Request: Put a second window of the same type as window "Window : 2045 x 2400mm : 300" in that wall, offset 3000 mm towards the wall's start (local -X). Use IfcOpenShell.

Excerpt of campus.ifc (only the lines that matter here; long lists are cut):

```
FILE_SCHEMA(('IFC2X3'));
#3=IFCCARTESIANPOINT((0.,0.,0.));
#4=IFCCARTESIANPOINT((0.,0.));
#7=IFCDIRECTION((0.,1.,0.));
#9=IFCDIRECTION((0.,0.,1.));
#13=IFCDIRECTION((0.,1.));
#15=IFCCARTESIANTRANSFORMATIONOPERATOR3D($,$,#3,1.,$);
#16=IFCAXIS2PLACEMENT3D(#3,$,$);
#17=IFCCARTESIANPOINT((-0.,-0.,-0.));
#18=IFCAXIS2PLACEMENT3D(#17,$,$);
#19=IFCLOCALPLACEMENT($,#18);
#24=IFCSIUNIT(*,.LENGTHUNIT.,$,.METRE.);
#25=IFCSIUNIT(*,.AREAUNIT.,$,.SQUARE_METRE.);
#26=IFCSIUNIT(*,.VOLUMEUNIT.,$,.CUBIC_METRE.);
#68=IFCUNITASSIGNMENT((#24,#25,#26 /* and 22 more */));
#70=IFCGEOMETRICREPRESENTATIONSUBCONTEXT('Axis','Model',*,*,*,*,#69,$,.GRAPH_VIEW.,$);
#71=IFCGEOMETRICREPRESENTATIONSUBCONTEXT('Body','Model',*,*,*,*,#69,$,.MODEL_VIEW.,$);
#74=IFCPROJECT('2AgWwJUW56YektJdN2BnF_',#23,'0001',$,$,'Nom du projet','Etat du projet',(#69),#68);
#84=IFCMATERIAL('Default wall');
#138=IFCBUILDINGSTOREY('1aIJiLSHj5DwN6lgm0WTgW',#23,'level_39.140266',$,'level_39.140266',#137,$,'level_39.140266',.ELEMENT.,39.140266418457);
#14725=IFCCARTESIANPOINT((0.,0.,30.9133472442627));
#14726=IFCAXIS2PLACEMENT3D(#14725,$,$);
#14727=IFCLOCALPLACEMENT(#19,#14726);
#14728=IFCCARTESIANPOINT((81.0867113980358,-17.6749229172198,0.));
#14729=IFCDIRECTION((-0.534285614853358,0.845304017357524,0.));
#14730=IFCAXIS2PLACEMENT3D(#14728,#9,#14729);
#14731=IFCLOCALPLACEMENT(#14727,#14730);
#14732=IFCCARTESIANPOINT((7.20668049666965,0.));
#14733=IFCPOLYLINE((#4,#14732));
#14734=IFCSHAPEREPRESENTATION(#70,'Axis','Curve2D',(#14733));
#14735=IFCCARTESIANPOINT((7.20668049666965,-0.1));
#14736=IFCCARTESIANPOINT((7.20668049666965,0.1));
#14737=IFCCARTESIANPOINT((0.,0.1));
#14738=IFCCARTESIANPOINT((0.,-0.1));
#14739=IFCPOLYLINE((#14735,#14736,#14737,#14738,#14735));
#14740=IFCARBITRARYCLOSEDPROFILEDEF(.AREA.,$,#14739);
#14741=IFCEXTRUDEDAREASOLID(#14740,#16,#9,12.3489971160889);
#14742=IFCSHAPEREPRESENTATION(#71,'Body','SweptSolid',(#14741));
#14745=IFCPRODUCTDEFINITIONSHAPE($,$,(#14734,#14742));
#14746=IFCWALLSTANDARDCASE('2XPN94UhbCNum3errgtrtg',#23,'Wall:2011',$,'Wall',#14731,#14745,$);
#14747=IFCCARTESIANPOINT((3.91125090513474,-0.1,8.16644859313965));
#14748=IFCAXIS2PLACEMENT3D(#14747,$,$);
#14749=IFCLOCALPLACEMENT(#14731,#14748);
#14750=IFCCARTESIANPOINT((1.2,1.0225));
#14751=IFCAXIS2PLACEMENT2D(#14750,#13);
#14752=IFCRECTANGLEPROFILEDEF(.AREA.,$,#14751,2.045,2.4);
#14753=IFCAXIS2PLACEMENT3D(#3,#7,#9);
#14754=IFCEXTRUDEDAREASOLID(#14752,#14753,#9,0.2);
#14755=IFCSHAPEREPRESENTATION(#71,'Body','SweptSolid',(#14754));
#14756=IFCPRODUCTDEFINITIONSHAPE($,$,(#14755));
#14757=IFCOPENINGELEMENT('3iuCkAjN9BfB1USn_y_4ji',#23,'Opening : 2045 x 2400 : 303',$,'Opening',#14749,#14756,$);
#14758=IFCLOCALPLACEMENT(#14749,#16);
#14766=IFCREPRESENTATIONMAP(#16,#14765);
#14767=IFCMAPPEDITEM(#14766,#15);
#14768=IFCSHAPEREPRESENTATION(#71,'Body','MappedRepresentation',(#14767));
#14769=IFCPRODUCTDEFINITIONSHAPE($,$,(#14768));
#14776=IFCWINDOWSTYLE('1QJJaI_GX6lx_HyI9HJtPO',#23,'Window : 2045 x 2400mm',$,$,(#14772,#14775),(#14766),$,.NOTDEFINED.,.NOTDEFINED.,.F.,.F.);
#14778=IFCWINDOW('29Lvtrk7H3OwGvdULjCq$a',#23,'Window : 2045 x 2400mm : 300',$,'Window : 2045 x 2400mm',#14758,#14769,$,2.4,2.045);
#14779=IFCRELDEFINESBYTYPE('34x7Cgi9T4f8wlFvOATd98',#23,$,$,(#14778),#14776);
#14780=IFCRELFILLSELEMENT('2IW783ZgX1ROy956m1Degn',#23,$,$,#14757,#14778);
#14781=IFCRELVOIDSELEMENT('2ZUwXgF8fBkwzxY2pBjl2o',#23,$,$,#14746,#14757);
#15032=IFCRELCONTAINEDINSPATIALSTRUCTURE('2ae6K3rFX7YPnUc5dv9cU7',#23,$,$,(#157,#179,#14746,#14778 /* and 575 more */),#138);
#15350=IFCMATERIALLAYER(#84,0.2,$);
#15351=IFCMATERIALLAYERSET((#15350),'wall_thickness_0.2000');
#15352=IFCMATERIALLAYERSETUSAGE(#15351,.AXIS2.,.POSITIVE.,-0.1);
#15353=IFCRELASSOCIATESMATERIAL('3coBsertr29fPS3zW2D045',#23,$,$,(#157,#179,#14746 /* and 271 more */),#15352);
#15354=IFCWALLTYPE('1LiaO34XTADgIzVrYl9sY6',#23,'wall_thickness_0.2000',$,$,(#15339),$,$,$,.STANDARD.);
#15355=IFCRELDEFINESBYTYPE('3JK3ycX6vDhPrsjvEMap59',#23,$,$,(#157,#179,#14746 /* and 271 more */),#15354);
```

```python
import ifcopenshell
import ifcopenshell.api.feature
import ifcopenshell.api.geometry
import ifcopenshell.api.root
import ifcopenshell.geom
import ifcopenshell.util.element
import ifcopenshell.util.placement
import ifcopenshell.util.shape
import ifcopenshell.util.unit

model = ifcopenshell.open("campus.ifc")
unit_scale = ifcopenshell.util.unit.calculate_unit_scale(model)
settings = ifcopenshell.geom.settings()


def volume(element):
    """Net volume in cubic metres, openings subtracted."""
    shape = ifcopenshell.geom.create_shape(settings, element)
    return ifcopenshell.util.shape.get_volume(shape.geometry)


window = model.by_guid("29Lvtrk7H3OwGvdULjCq$a")
opening = window.FillsVoids[0].RelatingOpeningElement
wall = opening.VoidsElements[0].RelatingBuildingElement
before = volume(wall)
shift = ifcopenshell.util.placement.get_local_placement(wall.ObjectPlacement)[:3, 0] * -3 / unit_scale

# copy_class copies the void relationship, type, container and properties, but no geometry.
new_opening = ifcopenshell.api.root.copy_class(model, product=opening)
new_opening.Representation = ifcopenshell.util.element.copy_deep(
    model, opening.Representation, exclude=["IfcGeometricRepresentationContext", "IfcRepresentationMap"]
)
new_opening.Name = "Opening : 2045 x 2400"
new_window = ifcopenshell.api.root.copy_class(model, product=window)
new_window.Representation = ifcopenshell.util.element.copy_deep(
    model, window.Representation, exclude=["IfcGeometricRepresentationContext", "IfcRepresentationMap"]
)
new_window.Name = "Window : 2045 x 2400mm"
fills = ifcopenshell.api.feature.add_filling(model, opening=new_opening, element=new_window)
fills.OwnerHistory = new_window.OwnerHistory  # required in IFC2X3

for old, new in ((opening, new_opening), (window, new_window)):
    matrix = ifcopenshell.util.placement.get_local_placement(old.ObjectPlacement)
    matrix[:3, 3] += shift
    ifcopenshell.api.geometry.edit_object_placement(model, product=new, matrix=matrix, is_si=False)

after = volume(wall)

print(f"wall volume {before:.3f} -> {after:.3f} m3")

model.write("campus_v2.ifc")
```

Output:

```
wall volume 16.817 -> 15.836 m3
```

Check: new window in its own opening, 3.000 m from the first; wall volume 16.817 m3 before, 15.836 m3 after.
